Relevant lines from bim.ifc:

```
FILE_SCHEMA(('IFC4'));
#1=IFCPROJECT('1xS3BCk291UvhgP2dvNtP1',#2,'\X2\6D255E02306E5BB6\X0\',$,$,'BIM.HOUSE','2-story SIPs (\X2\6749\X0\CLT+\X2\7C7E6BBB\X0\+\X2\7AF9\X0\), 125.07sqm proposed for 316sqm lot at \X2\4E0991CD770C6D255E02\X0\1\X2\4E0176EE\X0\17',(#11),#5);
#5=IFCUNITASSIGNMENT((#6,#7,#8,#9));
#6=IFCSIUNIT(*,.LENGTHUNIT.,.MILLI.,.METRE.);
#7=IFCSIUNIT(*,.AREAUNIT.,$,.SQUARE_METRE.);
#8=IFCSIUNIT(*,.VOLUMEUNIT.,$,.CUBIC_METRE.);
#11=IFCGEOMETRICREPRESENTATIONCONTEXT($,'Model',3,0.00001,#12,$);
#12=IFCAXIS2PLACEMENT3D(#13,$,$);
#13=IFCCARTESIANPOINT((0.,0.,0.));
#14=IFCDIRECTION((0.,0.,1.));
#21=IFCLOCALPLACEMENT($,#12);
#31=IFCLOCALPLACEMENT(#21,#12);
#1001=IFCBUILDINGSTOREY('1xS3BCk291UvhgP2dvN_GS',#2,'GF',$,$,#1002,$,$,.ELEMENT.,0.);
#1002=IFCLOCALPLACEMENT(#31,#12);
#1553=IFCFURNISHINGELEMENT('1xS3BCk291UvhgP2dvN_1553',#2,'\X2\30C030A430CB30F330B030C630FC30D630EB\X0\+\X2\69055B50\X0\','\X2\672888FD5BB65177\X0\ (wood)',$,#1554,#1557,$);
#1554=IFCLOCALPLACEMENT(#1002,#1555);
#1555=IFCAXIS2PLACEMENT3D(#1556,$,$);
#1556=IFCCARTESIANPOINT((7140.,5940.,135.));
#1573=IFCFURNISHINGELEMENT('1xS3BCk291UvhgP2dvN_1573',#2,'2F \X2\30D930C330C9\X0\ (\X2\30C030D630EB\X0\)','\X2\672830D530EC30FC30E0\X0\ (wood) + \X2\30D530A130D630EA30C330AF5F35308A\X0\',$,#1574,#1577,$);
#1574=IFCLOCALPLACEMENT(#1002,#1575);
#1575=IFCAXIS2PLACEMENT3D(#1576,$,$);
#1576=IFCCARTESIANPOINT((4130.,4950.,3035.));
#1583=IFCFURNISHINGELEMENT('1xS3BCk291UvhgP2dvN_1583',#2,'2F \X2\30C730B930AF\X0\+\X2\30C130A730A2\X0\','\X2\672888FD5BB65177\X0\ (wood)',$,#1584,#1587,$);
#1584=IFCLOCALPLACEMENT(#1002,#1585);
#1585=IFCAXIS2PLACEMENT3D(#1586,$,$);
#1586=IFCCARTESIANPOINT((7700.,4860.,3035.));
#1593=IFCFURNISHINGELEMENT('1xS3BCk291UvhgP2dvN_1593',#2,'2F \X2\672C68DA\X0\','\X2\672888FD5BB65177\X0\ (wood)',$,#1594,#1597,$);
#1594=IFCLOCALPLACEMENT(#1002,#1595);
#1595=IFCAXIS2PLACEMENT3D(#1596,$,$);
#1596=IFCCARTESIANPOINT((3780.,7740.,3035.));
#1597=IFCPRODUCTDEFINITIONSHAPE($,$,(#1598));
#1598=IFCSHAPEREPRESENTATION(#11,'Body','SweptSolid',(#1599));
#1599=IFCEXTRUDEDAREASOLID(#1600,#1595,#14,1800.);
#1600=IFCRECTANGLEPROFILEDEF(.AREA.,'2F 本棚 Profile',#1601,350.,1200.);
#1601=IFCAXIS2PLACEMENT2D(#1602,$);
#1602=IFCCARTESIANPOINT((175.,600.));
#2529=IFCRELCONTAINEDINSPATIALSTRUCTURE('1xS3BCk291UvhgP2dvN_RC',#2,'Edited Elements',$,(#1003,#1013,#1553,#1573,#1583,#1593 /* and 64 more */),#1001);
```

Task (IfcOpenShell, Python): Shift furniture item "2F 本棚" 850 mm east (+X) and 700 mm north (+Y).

```python
import ifcopenshell
import ifcopenshell.api.geometry
import ifcopenshell.util.placement
import ifcopenshell.util.unit

model = ifcopenshell.open("bim.ifc")
unit_scale = ifcopenshell.util.unit.calculate_unit_scale(model)

item = model.by_guid("1xS3BCk291UvhgP2dvN_1593")
matrix = ifcopenshell.util.placement.get_local_placement(item.ObjectPlacement)
matrix[0, 3] += 0.85 / unit_scale
matrix[1, 3] += 0.7 / unit_scale
ifcopenshell.api.geometry.edit_object_placement(model, product=item, matrix=matrix, is_si=False)

print(ifcopenshell.util.placement.get_local_placement(item.ObjectPlacement).round(3) + 0.0)

model.write("bim_rev.ifc")
```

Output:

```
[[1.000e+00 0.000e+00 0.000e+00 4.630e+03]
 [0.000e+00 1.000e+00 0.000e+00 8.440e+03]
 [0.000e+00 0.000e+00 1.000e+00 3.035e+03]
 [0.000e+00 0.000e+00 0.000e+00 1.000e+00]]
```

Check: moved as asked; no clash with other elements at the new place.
